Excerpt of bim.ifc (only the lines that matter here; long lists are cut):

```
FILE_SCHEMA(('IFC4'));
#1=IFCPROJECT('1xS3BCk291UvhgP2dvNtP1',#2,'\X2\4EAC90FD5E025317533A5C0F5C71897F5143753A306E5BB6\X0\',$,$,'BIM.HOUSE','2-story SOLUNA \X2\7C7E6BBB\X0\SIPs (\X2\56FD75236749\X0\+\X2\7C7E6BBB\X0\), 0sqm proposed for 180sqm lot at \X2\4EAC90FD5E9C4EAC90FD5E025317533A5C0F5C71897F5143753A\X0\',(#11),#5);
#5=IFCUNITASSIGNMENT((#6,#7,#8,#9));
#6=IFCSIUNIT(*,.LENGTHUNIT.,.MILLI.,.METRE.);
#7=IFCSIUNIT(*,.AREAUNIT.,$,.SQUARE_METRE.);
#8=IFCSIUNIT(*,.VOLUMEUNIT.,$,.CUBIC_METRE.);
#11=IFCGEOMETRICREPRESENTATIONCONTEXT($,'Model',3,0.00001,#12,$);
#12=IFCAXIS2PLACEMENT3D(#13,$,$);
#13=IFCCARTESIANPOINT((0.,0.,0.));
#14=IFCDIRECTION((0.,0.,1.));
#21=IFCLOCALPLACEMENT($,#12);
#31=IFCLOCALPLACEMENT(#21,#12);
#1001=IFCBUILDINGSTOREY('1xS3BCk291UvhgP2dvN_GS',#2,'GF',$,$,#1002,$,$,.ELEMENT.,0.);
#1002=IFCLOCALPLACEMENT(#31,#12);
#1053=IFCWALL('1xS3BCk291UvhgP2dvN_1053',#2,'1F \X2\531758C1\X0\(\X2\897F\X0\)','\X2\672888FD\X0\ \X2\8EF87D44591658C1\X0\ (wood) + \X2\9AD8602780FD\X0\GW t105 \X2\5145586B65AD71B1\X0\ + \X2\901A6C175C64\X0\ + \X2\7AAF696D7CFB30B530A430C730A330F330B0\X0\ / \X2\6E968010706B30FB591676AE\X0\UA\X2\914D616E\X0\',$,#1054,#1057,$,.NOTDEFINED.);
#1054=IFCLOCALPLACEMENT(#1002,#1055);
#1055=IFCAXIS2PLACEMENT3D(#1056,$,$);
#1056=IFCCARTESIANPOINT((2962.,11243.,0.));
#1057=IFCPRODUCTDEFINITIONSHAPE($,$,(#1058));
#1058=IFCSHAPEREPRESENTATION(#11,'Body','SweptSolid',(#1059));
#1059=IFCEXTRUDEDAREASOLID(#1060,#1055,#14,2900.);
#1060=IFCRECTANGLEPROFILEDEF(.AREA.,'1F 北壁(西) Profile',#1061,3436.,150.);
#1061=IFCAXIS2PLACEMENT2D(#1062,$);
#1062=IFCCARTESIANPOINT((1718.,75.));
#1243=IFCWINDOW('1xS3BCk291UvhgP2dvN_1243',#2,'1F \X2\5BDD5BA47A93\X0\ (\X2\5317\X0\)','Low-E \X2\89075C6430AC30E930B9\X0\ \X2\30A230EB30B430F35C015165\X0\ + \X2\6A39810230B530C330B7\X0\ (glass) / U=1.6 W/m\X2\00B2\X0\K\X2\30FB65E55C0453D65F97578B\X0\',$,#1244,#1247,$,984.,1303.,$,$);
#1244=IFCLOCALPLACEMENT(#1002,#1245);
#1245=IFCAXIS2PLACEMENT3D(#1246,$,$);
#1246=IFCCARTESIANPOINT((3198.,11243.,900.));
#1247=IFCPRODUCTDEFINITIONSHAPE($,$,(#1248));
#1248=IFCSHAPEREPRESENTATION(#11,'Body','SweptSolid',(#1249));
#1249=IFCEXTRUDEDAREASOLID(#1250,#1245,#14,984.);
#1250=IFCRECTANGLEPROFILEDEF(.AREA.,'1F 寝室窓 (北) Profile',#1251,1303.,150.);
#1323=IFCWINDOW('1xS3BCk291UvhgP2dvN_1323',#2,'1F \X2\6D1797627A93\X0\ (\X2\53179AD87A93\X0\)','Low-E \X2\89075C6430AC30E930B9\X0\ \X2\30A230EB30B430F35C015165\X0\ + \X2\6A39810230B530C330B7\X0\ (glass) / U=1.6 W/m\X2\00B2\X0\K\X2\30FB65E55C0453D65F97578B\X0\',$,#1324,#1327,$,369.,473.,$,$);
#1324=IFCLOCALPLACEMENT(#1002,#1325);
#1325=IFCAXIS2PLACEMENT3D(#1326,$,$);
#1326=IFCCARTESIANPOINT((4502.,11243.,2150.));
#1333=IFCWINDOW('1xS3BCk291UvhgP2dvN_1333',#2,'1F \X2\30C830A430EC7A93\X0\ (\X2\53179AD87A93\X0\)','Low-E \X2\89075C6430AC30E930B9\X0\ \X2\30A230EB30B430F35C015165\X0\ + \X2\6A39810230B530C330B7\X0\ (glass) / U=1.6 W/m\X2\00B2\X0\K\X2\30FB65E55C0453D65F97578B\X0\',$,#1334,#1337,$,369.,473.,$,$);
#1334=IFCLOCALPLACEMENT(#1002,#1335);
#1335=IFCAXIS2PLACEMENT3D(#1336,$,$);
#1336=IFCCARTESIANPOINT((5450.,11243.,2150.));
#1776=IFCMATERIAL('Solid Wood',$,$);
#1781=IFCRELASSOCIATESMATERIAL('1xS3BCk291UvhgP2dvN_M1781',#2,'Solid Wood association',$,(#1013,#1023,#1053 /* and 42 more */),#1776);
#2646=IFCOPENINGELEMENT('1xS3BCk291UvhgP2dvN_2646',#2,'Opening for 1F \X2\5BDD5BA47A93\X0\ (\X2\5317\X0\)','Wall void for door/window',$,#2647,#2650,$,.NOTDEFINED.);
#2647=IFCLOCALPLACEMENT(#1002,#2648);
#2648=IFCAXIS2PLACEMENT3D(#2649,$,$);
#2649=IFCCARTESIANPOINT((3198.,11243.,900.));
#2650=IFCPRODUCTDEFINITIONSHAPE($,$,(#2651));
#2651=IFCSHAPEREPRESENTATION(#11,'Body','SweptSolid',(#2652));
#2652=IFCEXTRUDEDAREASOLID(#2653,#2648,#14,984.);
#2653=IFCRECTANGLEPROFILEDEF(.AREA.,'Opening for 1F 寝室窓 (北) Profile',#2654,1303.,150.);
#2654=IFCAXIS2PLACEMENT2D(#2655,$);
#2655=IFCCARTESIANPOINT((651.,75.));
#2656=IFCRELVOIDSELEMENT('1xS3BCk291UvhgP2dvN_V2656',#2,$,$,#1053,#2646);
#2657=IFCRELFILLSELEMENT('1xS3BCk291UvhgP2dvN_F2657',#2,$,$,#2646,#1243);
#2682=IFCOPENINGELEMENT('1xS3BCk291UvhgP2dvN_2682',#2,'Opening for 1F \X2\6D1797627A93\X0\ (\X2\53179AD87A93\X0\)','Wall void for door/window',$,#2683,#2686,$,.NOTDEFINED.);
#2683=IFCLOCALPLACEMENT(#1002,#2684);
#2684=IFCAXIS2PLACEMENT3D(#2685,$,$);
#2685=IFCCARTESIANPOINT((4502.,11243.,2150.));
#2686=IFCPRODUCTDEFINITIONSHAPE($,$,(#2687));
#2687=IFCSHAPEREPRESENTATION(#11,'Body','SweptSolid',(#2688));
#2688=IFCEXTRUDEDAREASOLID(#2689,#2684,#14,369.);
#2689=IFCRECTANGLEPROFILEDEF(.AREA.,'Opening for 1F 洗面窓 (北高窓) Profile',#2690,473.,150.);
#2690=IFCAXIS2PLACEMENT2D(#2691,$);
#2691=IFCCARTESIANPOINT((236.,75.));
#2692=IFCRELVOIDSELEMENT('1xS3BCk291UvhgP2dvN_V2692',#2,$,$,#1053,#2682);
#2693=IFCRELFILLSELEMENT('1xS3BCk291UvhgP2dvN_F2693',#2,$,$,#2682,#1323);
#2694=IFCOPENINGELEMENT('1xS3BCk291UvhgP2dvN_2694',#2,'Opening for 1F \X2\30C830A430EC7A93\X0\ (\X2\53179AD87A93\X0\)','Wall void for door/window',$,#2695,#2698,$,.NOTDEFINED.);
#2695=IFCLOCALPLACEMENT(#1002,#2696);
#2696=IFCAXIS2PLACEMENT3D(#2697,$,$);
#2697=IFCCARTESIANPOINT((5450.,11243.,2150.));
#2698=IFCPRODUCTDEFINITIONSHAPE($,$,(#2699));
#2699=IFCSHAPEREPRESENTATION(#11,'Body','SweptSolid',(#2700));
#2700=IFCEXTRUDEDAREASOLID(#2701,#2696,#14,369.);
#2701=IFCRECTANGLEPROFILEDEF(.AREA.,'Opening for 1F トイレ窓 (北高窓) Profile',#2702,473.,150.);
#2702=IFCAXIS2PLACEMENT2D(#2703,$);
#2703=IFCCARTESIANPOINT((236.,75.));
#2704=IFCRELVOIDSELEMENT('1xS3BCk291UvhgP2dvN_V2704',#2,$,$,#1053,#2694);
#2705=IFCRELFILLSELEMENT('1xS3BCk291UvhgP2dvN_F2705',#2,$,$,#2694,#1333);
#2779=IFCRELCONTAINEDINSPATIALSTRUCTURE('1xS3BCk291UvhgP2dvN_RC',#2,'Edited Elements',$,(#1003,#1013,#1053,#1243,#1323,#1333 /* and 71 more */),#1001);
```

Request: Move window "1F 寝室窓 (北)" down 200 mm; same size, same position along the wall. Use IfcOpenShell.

```python
import numpy as np
import ifcopenshell
import ifcopenshell.api.geometry
import ifcopenshell.util.placement
import ifcopenshell.util.unit

model = ifcopenshell.open("bim.ifc")
unit_scale = ifcopenshell.util.unit.calculate_unit_scale(model)

window = model.by_guid("1xS3BCk291UvhgP2dvN_1243")
opening = window.FillsVoids[0].RelatingOpeningElement
dz = -0.2 / unit_scale

shift = np.array([0.0, 0.0, dz])
# The window is not placed relative to its opening, so move both.
for product in (opening, window):
    matrix = ifcopenshell.util.placement.get_local_placement(product.ObjectPlacement)
    matrix[:3, 3] += shift
    ifcopenshell.api.geometry.edit_object_placement(model, product=product, matrix=matrix, is_si=False)

print(f"moved by {dz * unit_scale:+.3f} m")

model.write("bim_edited.ifc")
```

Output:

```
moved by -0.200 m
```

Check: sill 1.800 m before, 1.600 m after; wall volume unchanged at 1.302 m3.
